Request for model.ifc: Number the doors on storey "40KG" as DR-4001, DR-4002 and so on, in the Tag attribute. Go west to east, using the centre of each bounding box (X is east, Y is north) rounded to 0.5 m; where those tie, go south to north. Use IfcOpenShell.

First a look at what the model holds.

```python
import ifcopenshell
import ifcopenshell.util.element
import ifcopenshell.util.placement

model = ifcopenshell.open("model.ifc")
print(model.schema)
storey = next(s for s in model.by_type("IfcBuildingStorey") if s.Name == "40KG")
doors = [e for e in ifcopenshell.util.element.get_decomposition(storey) if e.is_a("IfcDoor")]
for e in sorted(doors, key=lambda e: e.id()):
    origin = ifcopenshell.util.placement.get_local_placement(e.ObjectPlacement)[:3, 3]
    print(e.id(), e.Tag, e.Name, origin.round(2) + 0.0, sep=" | ")
```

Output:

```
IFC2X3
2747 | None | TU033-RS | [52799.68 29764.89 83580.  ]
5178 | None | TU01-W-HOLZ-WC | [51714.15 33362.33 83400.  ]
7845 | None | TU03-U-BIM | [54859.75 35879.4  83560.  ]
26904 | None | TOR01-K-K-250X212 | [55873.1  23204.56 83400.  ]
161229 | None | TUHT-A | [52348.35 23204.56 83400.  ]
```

```python
import ifcopenshell
import ifcopenshell.geom
import ifcopenshell.util.element
import ifcopenshell.util.shape

model = ifcopenshell.open("model.ifc")
settings = ifcopenshell.geom.settings()
settings.set("use-world-coords", True)


def centre(element):
    shape = ifcopenshell.geom.create_shape(settings, element)
    return ifcopenshell.util.shape.get_bbox_centroid(shape.geometry)


storey = next(s for s in model.by_type("IfcBuildingStorey") if s.Name == "40KG")
doors = [e for e in ifcopenshell.util.element.get_decomposition(storey) if e.is_a("IfcDoor")]

# Insertion points can sit at a corner or the storey origin, so sort by the geometry (in metres).
centres = {e: centre(e) for e in doors}
doors.sort(key=lambda e: (round(centres[e][0] / 0.5), centres[e][1]))

for i, e in enumerate(doors, start=1):
    number = f"DR-40{i:02d}"
    e.Tag = number
    print(e.id(), number)

model.write("model-out.ifc")
```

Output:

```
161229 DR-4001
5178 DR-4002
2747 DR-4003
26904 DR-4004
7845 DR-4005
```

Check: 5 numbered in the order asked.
